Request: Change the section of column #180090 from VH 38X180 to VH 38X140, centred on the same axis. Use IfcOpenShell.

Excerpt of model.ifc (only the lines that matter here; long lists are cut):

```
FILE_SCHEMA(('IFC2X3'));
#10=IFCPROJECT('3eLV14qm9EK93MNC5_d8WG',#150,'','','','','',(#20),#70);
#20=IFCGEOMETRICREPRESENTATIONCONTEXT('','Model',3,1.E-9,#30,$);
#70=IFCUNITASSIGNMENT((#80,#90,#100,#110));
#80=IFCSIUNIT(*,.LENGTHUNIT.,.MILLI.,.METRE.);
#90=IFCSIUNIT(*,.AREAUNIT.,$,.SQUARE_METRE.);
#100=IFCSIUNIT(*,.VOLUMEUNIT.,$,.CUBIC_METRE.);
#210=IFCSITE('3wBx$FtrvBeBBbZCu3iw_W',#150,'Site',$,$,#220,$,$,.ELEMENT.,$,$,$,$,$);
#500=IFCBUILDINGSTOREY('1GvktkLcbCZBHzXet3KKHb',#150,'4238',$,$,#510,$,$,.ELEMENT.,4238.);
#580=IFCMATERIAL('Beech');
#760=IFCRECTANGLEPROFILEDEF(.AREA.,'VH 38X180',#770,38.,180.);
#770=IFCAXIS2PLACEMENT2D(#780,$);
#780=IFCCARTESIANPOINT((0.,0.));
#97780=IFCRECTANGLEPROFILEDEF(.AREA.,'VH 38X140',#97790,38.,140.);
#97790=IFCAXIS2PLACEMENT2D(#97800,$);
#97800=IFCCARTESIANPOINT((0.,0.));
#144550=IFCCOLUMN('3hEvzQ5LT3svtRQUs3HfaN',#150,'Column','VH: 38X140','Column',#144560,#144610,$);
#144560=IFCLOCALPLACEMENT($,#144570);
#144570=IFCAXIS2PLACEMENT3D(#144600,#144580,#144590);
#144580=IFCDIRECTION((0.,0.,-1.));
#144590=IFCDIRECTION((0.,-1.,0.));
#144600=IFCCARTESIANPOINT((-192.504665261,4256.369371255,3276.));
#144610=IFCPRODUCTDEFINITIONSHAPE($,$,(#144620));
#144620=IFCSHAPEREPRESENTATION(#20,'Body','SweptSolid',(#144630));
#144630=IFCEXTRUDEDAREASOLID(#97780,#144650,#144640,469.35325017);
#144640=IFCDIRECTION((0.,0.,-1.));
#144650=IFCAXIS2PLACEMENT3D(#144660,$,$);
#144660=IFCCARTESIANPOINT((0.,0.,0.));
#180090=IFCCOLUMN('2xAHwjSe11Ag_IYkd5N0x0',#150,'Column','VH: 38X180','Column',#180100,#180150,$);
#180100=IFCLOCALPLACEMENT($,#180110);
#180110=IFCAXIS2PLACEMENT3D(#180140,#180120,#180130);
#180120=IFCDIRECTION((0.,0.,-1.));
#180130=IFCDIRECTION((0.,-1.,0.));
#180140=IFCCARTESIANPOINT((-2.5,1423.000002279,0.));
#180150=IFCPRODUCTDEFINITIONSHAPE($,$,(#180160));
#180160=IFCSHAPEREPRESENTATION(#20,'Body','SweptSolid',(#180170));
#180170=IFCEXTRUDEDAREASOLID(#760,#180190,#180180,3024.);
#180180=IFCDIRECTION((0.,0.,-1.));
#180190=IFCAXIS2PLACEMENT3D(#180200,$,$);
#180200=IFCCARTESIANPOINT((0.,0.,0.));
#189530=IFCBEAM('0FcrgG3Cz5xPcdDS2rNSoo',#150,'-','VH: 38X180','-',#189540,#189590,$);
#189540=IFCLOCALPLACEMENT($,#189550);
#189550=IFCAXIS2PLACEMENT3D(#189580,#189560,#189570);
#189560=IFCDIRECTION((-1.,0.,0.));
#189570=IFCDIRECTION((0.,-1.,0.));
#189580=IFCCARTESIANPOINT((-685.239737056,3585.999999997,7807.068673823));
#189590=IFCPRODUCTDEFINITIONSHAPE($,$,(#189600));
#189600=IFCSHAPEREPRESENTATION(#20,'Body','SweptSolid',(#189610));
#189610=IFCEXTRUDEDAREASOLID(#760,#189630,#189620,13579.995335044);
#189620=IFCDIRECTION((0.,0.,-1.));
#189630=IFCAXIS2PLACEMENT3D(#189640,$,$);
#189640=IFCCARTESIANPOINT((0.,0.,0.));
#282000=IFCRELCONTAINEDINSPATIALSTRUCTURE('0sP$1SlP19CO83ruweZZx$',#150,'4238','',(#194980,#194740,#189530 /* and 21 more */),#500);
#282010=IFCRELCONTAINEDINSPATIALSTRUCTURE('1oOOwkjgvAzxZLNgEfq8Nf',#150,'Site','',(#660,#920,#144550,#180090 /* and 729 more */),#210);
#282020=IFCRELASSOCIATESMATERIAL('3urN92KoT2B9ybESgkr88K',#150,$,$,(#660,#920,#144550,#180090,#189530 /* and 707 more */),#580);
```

```python
import ifcopenshell
import ifcopenshell.util.element

model = ifcopenshell.open("model.ifc")

member = model.by_guid("2xAHwjSe11Ag_IYkd5N0x0")
source = next(p for p in model.by_type("IfcRectangleProfileDef") if p.ProfileName == "VH 38X140")

body = next(r for r in member.Representation.Representations if r.RepresentationIdentifier == "Body")
solid = body.Items[0]
old_profile = solid.SweptArea

# Copy the section's sizes but keep this member's own profile position.
profile = ifcopenshell.util.element.copy(model, source)
profile.Position = old_profile.Position
solid.SweptArea = profile
if not model.get_total_inverses(old_profile):
    ifcopenshell.util.element.remove_deep2(model, old_profile)

print(solid.SweptArea)

model.write("model_edited.ifc")
```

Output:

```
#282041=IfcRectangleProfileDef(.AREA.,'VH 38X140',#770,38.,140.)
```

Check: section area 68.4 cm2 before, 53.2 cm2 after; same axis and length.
